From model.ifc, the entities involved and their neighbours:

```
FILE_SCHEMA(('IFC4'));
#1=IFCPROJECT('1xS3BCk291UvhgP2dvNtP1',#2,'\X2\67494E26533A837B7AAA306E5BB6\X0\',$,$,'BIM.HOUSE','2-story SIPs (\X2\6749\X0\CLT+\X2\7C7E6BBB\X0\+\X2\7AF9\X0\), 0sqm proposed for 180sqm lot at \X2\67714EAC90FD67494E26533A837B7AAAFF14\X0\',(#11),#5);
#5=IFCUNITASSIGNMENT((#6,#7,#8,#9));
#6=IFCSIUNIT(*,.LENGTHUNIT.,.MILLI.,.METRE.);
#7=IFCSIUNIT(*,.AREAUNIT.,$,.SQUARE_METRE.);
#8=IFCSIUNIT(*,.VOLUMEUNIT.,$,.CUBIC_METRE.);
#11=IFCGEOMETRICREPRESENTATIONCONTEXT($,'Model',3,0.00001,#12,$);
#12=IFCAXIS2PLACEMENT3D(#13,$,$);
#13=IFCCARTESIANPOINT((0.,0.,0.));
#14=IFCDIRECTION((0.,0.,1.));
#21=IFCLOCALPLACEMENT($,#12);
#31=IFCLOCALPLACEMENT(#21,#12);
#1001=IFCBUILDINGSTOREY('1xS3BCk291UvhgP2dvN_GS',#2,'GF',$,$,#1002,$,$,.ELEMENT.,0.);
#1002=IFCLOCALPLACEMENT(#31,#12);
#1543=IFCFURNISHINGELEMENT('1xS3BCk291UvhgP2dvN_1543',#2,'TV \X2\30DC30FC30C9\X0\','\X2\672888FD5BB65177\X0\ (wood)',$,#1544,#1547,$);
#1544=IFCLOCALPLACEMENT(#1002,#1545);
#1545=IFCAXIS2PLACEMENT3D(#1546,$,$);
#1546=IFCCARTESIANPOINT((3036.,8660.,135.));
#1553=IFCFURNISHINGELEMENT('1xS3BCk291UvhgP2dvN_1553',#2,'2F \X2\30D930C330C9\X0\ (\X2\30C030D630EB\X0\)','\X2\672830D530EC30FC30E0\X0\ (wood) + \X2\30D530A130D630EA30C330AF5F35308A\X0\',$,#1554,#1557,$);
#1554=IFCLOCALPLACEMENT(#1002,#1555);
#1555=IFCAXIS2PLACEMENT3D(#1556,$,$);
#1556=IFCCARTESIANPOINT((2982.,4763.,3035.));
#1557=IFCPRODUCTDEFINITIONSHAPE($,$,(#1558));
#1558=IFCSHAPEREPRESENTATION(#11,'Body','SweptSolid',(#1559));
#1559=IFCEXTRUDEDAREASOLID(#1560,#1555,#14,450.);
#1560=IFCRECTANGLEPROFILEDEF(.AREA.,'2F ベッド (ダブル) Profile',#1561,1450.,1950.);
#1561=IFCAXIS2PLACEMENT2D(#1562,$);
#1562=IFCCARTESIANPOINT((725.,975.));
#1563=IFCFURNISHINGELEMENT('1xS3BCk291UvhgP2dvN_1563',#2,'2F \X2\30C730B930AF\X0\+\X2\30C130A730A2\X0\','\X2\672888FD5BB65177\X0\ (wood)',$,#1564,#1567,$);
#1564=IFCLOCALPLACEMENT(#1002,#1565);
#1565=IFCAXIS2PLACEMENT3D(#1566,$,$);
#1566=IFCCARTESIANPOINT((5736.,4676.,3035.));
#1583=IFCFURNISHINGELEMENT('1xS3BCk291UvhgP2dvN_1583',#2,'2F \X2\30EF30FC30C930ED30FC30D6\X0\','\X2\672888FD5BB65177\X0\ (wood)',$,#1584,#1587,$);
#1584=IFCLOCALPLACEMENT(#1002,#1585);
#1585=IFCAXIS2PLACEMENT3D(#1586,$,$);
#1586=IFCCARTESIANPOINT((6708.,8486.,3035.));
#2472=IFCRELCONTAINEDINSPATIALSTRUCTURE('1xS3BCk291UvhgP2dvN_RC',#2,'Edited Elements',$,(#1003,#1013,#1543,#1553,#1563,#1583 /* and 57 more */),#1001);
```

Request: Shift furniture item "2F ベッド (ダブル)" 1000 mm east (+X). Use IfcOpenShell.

```python
import ifcopenshell
import ifcopenshell.api.geometry
import ifcopenshell.util.placement
import ifcopenshell.util.unit

model = ifcopenshell.open("model.ifc")
unit_scale = ifcopenshell.util.unit.calculate_unit_scale(model)

item = model.by_guid("1xS3BCk291UvhgP2dvN_1553")
matrix = ifcopenshell.util.placement.get_local_placement(item.ObjectPlacement)
matrix[0, 3] += 1 / unit_scale
ifcopenshell.api.geometry.edit_object_placement(model, product=item, matrix=matrix, is_si=False)

print(ifcopenshell.util.placement.get_local_placement(item.ObjectPlacement).round(3) + 0.0)

model.write("model_updated.ifc")
```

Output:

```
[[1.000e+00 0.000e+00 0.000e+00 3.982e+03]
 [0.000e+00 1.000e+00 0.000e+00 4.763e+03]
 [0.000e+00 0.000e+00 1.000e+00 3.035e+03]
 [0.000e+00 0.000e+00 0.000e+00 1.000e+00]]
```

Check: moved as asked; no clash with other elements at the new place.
